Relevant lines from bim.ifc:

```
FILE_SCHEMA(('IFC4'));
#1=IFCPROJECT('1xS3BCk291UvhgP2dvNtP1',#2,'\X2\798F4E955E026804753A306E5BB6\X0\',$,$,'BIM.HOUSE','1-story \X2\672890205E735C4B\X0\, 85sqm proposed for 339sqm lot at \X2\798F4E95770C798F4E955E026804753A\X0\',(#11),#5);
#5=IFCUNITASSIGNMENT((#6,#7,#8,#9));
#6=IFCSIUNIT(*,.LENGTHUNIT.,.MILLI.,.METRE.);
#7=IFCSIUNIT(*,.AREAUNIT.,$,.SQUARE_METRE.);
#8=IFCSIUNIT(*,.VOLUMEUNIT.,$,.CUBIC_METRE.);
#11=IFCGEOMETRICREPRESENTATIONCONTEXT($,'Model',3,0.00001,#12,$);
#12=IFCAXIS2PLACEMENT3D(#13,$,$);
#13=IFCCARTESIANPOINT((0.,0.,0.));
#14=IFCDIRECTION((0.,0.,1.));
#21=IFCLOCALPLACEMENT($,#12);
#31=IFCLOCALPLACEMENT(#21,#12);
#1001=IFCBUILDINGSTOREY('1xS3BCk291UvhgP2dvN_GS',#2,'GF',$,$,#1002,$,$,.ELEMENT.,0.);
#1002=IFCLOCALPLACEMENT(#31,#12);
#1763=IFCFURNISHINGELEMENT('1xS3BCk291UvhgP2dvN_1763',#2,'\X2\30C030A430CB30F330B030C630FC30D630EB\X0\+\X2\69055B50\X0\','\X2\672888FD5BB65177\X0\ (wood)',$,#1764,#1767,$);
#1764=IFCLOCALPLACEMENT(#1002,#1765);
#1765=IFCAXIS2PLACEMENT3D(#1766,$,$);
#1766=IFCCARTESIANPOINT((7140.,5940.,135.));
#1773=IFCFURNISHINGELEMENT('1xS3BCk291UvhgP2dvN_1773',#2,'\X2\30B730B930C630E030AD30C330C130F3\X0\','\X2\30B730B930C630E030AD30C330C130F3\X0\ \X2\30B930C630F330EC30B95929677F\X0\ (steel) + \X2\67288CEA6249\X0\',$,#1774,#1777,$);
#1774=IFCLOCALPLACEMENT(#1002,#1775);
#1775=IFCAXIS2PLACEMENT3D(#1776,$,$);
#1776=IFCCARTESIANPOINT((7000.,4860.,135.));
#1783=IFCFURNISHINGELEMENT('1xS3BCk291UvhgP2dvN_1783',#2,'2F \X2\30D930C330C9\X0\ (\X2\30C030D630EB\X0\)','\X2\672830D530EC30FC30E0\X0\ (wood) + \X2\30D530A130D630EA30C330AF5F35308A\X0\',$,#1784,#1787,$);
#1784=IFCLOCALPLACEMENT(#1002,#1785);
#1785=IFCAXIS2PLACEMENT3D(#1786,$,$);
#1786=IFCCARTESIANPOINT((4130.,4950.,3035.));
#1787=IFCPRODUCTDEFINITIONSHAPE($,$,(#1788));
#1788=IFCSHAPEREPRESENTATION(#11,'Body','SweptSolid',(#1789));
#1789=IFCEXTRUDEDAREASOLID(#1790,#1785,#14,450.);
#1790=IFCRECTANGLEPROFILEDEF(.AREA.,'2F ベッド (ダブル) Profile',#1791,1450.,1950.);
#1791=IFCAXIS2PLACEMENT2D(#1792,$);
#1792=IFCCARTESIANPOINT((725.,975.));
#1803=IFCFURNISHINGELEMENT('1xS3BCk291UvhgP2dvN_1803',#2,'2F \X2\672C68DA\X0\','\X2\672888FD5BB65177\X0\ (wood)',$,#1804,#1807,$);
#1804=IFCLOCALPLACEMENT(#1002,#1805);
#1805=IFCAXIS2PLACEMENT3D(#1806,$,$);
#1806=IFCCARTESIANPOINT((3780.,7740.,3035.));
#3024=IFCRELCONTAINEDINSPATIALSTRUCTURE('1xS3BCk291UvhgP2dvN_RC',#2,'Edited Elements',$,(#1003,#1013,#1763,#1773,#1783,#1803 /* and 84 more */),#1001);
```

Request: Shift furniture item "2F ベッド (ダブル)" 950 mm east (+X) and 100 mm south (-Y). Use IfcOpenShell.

```python
import ifcopenshell
import ifcopenshell.api.geometry
import ifcopenshell.util.placement
import ifcopenshell.util.unit

model = ifcopenshell.open("bim.ifc")
unit_scale = ifcopenshell.util.unit.calculate_unit_scale(model)

item = model.by_guid("1xS3BCk291UvhgP2dvN_1783")
matrix = ifcopenshell.util.placement.get_local_placement(item.ObjectPlacement)
matrix[0, 3] += 0.95 / unit_scale
matrix[1, 3] -= 0.1 / unit_scale
ifcopenshell.api.geometry.edit_object_placement(model, product=item, matrix=matrix, is_si=False)

print(ifcopenshell.util.placement.get_local_placement(item.ObjectPlacement).round(3) + 0.0)

model.write("bim_edited.ifc")
```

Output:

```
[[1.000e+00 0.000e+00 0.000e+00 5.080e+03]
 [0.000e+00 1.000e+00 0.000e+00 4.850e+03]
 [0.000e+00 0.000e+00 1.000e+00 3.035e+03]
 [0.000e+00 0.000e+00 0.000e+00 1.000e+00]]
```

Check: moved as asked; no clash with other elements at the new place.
